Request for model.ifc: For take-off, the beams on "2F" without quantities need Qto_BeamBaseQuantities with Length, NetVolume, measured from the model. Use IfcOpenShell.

First a look at what the model holds.

```python
import ifcopenshell
import ifcopenshell.util.element
import ifcopenshell.util.unit

model = ifcopenshell.open("model.ifc")
print(model.schema)
for unit_type in ("LENGTHUNIT", "AREAUNIT", "VOLUMEUNIT"):
    print(unit_type, ifcopenshell.util.unit.calculate_unit_scale(model, unit_type))
storey = next(s for s in model.by_type("IfcBuildingStorey") if s.Name == "2F")
beams = [e for e in ifcopenshell.util.element.get_decomposition(storey) if e.is_a("IfcBeam")]
for e in sorted(beams, key=lambda e: e.id()):
    print(e.id(), e.is_a(), e.Name, list(ifcopenshell.util.element.get_psets(e, qtos_only=True)), sep=" | ")
```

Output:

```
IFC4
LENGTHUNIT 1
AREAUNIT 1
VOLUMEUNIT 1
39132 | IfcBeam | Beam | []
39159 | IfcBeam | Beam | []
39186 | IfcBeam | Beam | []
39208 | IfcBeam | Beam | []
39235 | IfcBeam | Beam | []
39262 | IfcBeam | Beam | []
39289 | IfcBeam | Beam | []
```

```python
import ifcopenshell
import ifcopenshell.api.pset
import ifcopenshell.geom
import ifcopenshell.util.element
import ifcopenshell.util.shape
import ifcopenshell.util.unit

model = ifcopenshell.open("model.ifc")
unit_scale = ifcopenshell.util.unit.calculate_unit_scale(model)
volume_scale = ifcopenshell.util.unit.calculate_unit_scale(model, "VOLUMEUNIT")
settings = ifcopenshell.geom.settings()

storey = next(s for s in model.by_type("IfcBuildingStorey") if s.Name == "2F")
beams = [e for e in ifcopenshell.util.element.get_decomposition(storey) if e.is_a("IfcBeam")]

for e in sorted(beams, key=lambda e: e.id()):
    if ifcopenshell.util.element.get_psets(e, qtos_only=True, should_inherit=False):
        continue
    # Geometry comes back in metres, in the element's own axes.
    shape = ifcopenshell.geom.create_shape(settings, e)
    values = {
        "Length": ifcopenshell.util.shape.get_max_xyz(shape.geometry) / unit_scale,
        "NetVolume": ifcopenshell.util.shape.get_volume(shape.geometry) / volume_scale,
    }
    qto = ifcopenshell.api.pset.add_qto(model, product=e, name="Qto_BeamBaseQuantities")
    ifcopenshell.api.pset.edit_qto(model, qto=qto, properties=values)
    print(e.id(), {k: round(v, 3) for k, v in values.items()})

model.write("model_edited.ifc")
```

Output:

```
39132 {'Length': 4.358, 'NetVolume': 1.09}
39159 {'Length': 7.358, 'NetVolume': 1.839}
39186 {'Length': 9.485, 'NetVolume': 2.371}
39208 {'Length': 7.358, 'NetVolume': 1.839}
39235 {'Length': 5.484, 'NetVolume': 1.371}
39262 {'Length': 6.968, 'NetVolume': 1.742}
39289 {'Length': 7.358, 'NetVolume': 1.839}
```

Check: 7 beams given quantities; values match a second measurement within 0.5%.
